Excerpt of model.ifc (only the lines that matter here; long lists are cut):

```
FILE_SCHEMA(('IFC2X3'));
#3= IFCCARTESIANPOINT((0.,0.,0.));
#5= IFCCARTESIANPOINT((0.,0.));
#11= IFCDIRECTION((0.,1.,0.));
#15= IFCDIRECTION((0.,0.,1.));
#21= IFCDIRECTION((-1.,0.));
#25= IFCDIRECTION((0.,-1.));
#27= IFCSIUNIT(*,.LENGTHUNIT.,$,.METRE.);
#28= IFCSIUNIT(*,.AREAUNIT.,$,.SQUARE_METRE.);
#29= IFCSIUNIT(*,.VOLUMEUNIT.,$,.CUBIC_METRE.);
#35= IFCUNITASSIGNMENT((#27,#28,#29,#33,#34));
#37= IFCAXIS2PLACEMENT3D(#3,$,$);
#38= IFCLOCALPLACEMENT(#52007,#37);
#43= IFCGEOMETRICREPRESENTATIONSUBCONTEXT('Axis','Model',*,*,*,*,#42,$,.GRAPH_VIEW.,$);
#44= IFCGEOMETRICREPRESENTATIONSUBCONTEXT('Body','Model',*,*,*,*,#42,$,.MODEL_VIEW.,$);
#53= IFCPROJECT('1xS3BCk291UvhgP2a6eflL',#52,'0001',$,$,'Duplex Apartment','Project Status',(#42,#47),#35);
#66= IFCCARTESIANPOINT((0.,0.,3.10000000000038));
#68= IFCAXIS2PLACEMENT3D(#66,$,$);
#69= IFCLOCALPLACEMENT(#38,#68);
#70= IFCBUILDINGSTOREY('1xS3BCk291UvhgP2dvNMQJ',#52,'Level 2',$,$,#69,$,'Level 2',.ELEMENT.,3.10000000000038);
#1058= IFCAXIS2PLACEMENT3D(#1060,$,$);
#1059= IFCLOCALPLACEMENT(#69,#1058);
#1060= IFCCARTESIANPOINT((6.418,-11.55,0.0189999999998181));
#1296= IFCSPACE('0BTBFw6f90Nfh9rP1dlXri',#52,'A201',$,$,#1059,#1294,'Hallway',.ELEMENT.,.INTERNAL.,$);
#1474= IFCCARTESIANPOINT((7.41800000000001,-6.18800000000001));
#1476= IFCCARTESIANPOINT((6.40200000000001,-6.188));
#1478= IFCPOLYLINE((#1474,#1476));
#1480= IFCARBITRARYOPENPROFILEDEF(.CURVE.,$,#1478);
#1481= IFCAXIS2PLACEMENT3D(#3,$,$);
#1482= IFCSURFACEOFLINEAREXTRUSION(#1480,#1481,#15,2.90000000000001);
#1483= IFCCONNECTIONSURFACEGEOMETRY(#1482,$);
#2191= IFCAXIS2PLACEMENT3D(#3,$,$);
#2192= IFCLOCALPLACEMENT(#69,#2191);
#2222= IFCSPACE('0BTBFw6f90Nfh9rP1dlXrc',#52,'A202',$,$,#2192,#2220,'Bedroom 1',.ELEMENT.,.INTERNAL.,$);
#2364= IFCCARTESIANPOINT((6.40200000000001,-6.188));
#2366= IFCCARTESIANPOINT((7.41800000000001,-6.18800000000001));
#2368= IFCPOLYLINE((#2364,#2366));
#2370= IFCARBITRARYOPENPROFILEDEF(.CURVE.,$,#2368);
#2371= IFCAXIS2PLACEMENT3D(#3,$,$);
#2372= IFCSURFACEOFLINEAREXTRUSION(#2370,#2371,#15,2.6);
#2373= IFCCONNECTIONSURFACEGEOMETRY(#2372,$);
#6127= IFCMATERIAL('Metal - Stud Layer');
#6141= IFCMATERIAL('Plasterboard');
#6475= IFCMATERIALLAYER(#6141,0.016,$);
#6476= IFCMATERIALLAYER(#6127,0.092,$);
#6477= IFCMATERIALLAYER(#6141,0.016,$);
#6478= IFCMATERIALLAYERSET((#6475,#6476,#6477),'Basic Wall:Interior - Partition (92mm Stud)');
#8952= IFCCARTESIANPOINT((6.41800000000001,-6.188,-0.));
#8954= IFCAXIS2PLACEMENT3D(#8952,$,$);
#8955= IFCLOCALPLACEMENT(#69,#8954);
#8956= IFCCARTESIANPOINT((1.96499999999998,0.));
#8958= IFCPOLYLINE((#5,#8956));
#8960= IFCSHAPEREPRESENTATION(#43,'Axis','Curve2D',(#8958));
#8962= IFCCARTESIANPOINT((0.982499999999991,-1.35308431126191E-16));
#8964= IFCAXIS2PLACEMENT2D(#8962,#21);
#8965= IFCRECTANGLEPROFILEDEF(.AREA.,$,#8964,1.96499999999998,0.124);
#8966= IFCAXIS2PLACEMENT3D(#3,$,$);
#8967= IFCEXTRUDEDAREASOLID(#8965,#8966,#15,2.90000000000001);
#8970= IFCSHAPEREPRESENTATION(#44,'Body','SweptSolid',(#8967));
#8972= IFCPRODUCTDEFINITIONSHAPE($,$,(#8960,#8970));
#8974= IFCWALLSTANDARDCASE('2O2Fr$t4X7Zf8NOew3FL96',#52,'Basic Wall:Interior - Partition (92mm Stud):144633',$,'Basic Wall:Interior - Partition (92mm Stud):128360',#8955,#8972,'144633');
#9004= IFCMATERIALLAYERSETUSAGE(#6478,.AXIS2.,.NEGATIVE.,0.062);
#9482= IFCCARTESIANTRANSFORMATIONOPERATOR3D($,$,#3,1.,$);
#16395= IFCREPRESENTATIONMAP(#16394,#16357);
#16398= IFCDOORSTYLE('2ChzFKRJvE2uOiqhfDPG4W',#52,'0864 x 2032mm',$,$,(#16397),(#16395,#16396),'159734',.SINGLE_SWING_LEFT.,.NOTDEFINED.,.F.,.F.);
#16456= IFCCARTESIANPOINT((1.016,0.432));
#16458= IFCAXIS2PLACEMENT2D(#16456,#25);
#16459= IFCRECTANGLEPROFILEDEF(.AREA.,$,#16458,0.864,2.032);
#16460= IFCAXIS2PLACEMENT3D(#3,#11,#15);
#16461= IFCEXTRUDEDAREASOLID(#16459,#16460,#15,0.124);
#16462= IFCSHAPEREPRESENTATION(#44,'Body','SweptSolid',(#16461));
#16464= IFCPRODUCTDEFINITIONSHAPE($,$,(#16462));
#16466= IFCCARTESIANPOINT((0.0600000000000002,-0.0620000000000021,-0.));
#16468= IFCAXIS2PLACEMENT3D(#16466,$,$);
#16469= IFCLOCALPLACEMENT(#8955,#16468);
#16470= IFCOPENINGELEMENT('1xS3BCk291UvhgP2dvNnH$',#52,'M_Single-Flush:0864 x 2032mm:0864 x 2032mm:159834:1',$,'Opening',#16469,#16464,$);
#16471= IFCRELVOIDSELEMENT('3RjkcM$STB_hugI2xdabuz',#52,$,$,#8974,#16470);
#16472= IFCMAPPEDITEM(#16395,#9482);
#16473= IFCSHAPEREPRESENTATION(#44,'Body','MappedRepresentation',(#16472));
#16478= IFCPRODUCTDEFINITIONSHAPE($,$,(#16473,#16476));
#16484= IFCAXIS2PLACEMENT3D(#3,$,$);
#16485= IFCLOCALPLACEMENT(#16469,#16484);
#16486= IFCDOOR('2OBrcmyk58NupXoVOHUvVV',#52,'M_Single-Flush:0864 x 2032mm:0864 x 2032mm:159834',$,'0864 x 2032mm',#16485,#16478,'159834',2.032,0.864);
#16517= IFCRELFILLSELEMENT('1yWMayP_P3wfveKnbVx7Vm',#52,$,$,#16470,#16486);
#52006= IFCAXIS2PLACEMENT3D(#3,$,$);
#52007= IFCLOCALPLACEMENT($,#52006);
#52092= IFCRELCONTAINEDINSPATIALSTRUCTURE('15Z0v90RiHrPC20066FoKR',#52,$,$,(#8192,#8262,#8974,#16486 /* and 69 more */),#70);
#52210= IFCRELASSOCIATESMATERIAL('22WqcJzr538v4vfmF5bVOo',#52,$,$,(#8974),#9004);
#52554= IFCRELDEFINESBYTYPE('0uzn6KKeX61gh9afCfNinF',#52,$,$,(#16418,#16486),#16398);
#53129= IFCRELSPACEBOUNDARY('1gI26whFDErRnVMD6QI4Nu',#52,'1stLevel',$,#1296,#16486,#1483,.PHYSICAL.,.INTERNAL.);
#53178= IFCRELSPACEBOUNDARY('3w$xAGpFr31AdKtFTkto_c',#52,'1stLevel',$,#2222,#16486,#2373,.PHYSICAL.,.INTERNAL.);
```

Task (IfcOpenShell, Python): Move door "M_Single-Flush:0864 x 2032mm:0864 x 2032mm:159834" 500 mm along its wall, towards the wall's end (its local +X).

```python
import numpy as np
import ifcopenshell
import ifcopenshell.api.geometry
import ifcopenshell.util.placement
import ifcopenshell.util.unit

model = ifcopenshell.open("model.ifc")
unit_scale = ifcopenshell.util.unit.calculate_unit_scale(model)

door = model.by_guid("2OBrcmyk58NupXoVOHUvVV")
opening = door.FillsVoids[0].RelatingOpeningElement
wall = opening.VoidsElements[0].RelatingBuildingElement

wall_matrix = ifcopenshell.util.placement.get_local_placement(wall.ObjectPlacement)
shift = wall_matrix[:3, 0] * 0.5 / unit_scale
before = ifcopenshell.util.placement.get_local_placement(door.ObjectPlacement)[:3, 3].copy()

# The door is placed relative to its opening, so it follows when the opening moves.
matrix = ifcopenshell.util.placement.get_local_placement(opening.ObjectPlacement)
matrix[:3, 3] += shift
ifcopenshell.api.geometry.edit_object_placement(
    model, product=opening, matrix=matrix, is_si=False, should_transform_children=True
)

# Space boundary surfaces are stored in each space's coordinates; move them too.
for rel in door.ProvidesBoundaries:
    if not rel.ConnectionGeometry:
        continue
    surface = rel.ConnectionGeometry.SurfaceOnRelatingElement
    space_matrix = ifcopenshell.util.placement.get_local_placement(rel.RelatingSpace.ObjectPlacement)
    point = np.array(surface.Position.Location.Coordinates) + space_matrix[:3, :3].T @ shift
    surface.Position = model.createIfcAxis2Placement3D(
        model.createIfcCartesianPoint(point.tolist()), surface.Position.Axis, surface.Position.RefDirection
    )

after = ifcopenshell.util.placement.get_local_placement(door.ObjectPlacement)[:3, 3]
print("door moved by", (after - before).round(3) + 0.0)

model.write("model_updated.ifc")
```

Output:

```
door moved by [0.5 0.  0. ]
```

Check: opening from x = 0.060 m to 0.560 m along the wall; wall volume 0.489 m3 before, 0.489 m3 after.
